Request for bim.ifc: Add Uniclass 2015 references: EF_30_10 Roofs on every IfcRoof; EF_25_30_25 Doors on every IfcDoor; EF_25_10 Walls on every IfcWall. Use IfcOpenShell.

First a look at what the model holds.

```python
import ifcopenshell

model = ifcopenshell.open("bim.ifc")
print(model.schema)
print("classifications:", [c.Name for c in model.by_type("IfcClassification")])
for ifc_class in ("IfcDoor", "IfcRoof", "IfcStair", "IfcWall", "IfcWindow"):
    print(ifc_class, len(model.by_type(ifc_class)))
```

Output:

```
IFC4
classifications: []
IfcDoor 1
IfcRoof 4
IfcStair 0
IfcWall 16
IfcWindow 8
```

```python
import ifcopenshell
import ifcopenshell.api.classification

model = ifcopenshell.open("bim.ifc")

system = ifcopenshell.api.classification.add_classification(model, classification="Uniclass 2015")

codes = {
    "IfcRoof": ("EF_30_10", "Roofs"),
    "IfcDoor": ("EF_25_30_25", "Doors"),
    "IfcWall": ("EF_25_10", "Walls"),
}
for ifc_class, (code, name) in codes.items():
    products = model.by_type(ifc_class)
    ifcopenshell.api.classification.add_reference(
        model, products=products, classification=system, identification=code, name=name
    )
    print(code, len(products))

model.write("bim_updated.ifc")
```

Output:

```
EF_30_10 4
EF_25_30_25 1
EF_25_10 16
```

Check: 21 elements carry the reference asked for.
